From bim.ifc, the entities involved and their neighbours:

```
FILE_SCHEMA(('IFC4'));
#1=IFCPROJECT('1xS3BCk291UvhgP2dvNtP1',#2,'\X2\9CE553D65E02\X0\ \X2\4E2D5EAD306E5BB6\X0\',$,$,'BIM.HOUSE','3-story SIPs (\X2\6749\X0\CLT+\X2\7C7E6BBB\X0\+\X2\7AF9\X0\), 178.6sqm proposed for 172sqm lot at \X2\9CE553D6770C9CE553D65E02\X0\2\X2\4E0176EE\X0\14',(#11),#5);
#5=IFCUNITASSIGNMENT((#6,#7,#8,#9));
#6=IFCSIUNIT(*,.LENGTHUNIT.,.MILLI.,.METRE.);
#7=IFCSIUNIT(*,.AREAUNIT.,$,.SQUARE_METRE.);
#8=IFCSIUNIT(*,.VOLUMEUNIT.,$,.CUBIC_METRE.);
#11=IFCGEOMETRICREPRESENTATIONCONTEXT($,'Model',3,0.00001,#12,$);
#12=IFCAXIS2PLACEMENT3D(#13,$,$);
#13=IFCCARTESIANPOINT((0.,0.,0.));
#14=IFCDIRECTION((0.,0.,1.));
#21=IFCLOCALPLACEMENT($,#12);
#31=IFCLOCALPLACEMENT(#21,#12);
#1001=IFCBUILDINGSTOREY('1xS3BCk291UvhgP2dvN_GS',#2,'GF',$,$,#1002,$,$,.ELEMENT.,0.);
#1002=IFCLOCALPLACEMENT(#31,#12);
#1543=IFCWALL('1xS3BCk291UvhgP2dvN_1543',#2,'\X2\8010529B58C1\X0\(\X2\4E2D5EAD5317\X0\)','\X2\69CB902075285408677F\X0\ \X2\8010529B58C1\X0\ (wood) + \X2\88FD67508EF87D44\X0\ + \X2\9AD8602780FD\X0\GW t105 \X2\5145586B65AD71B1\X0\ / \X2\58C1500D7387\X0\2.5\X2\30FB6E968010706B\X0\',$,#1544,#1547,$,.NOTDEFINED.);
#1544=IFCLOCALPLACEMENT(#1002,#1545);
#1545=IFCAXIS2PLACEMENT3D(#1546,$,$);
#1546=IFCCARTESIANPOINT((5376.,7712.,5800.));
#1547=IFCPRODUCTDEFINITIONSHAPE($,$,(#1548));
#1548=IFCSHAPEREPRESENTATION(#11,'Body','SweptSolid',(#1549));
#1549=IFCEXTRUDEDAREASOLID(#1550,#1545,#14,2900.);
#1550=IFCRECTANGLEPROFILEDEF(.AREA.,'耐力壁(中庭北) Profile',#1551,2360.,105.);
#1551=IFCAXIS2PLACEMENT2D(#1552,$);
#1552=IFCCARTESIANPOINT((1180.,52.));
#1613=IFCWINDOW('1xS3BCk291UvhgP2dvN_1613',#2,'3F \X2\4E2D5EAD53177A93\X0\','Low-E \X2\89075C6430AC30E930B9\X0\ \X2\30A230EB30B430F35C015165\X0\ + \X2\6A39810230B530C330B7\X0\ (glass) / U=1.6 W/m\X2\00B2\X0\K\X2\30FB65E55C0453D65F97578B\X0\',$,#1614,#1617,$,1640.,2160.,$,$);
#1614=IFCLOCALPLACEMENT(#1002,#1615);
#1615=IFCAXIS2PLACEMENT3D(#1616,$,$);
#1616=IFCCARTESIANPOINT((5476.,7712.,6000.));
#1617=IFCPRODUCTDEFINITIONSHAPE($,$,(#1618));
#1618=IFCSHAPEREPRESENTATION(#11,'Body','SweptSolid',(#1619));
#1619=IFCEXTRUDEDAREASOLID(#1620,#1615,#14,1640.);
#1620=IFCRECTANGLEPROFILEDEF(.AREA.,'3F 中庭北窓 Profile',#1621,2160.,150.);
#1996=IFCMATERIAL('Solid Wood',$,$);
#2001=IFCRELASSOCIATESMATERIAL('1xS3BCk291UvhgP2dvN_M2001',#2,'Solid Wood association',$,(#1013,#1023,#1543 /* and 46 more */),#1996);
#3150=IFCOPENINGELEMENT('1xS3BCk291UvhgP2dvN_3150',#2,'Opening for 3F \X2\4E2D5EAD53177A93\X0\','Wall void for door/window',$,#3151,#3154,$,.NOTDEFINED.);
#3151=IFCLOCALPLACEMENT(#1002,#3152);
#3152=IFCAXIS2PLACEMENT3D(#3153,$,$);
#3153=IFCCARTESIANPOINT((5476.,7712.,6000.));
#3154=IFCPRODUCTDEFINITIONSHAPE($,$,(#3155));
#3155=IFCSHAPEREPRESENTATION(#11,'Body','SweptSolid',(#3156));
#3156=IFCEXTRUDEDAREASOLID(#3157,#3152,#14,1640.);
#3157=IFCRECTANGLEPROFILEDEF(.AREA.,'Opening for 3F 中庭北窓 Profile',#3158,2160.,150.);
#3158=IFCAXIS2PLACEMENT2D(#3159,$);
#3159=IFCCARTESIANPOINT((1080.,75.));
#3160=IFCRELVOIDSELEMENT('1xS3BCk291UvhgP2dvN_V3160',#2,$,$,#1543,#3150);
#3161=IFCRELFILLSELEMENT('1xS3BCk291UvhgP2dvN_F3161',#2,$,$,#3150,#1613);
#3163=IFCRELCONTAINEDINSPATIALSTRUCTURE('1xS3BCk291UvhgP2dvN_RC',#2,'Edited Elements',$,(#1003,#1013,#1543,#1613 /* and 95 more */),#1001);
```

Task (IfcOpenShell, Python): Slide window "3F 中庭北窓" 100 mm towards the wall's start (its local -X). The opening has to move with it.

```python
import ifcopenshell
import ifcopenshell.api.geometry
import ifcopenshell.util.placement
import ifcopenshell.util.unit

model = ifcopenshell.open("bim.ifc")
unit_scale = ifcopenshell.util.unit.calculate_unit_scale(model)

window = model.by_id(1613)
opening = window.FillsVoids[0].RelatingOpeningElement
wall = opening.VoidsElements[0].RelatingBuildingElement

wall_matrix = ifcopenshell.util.placement.get_local_placement(wall.ObjectPlacement)
shift = wall_matrix[:3, 0] * -0.1 / unit_scale
before = ifcopenshell.util.placement.get_local_placement(window.ObjectPlacement)[:3, 3].copy()

# The window is not placed relative to its opening, so move both.
for product in (opening, window):
    matrix = ifcopenshell.util.placement.get_local_placement(product.ObjectPlacement)
    matrix[:3, 3] += shift
    ifcopenshell.api.geometry.edit_object_placement(model, product=product, matrix=matrix, is_si=False)

after = ifcopenshell.util.placement.get_local_placement(window.ObjectPlacement)[:3, 3]
print("window moved by", (after - before).round(3) + 0.0)

model.write("bim_v2.ifc")
```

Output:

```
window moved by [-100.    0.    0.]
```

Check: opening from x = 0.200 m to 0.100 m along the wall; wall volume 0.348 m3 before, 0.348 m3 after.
